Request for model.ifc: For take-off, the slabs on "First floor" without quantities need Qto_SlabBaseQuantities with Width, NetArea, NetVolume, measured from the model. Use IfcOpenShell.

First a look at what the model holds.

```python
import ifcopenshell
import ifcopenshell.util.element
import ifcopenshell.util.unit

model = ifcopenshell.open("model.ifc")
print(model.schema)
for unit_type in ("LENGTHUNIT", "AREAUNIT", "VOLUMEUNIT"):
    print(unit_type, ifcopenshell.util.unit.calculate_unit_scale(model, unit_type))
storey = next(s for s in model.by_type("IfcBuildingStorey") if s.Name == "First floor")
slabs = [e for e in ifcopenshell.util.element.get_decomposition(storey) if e.is_a("IfcSlab")]
for e in sorted(slabs, key=lambda e: e.id()):
    print(e.id(), e.is_a(), e.Name, list(ifcopenshell.util.element.get_psets(e, qtos_only=True)), sep=" | ")
```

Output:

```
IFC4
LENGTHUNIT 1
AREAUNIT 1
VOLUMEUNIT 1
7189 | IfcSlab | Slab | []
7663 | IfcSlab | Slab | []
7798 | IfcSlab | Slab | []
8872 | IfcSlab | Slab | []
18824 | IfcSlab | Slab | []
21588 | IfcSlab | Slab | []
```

```python
import ifcopenshell
import ifcopenshell.api.pset
import ifcopenshell.geom
import ifcopenshell.util.element
import ifcopenshell.util.shape
import ifcopenshell.util.unit

model = ifcopenshell.open("model.ifc")
unit_scale = ifcopenshell.util.unit.calculate_unit_scale(model)
area_scale = ifcopenshell.util.unit.calculate_unit_scale(model, "AREAUNIT")
volume_scale = ifcopenshell.util.unit.calculate_unit_scale(model, "VOLUMEUNIT")
settings = ifcopenshell.geom.settings()

storey = next(s for s in model.by_type("IfcBuildingStorey") if s.Name == "First floor")
slabs = [e for e in ifcopenshell.util.element.get_decomposition(storey) if e.is_a("IfcSlab")]

for e in sorted(slabs, key=lambda e: e.id()):
    if ifcopenshell.util.element.get_psets(e, qtos_only=True, should_inherit=False):
        continue
    # Geometry comes back in metres, in the element's own axes.
    shape = ifcopenshell.geom.create_shape(settings, e)
    values = {
        "Width": ifcopenshell.util.shape.get_z(shape.geometry) / unit_scale,
        "NetArea": ifcopenshell.util.shape.get_footprint_area(shape.geometry) / area_scale,
        "NetVolume": ifcopenshell.util.shape.get_volume(shape.geometry) / volume_scale,
    }
    qto = ifcopenshell.api.pset.add_qto(model, product=e, name="Qto_SlabBaseQuantities")
    ifcopenshell.api.pset.edit_qto(model, qto=qto, properties=values)
    print(e.id(), {k: round(v, 3) for k, v in values.items()})

model.write("model_v2.ifc")
```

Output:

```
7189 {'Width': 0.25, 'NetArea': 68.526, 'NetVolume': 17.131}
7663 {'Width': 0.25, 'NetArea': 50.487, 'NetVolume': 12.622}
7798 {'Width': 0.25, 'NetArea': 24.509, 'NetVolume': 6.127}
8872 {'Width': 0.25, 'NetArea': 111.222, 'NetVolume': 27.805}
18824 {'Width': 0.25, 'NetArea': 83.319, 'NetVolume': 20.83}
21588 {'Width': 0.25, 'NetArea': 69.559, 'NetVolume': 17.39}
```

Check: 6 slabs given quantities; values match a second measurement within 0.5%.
